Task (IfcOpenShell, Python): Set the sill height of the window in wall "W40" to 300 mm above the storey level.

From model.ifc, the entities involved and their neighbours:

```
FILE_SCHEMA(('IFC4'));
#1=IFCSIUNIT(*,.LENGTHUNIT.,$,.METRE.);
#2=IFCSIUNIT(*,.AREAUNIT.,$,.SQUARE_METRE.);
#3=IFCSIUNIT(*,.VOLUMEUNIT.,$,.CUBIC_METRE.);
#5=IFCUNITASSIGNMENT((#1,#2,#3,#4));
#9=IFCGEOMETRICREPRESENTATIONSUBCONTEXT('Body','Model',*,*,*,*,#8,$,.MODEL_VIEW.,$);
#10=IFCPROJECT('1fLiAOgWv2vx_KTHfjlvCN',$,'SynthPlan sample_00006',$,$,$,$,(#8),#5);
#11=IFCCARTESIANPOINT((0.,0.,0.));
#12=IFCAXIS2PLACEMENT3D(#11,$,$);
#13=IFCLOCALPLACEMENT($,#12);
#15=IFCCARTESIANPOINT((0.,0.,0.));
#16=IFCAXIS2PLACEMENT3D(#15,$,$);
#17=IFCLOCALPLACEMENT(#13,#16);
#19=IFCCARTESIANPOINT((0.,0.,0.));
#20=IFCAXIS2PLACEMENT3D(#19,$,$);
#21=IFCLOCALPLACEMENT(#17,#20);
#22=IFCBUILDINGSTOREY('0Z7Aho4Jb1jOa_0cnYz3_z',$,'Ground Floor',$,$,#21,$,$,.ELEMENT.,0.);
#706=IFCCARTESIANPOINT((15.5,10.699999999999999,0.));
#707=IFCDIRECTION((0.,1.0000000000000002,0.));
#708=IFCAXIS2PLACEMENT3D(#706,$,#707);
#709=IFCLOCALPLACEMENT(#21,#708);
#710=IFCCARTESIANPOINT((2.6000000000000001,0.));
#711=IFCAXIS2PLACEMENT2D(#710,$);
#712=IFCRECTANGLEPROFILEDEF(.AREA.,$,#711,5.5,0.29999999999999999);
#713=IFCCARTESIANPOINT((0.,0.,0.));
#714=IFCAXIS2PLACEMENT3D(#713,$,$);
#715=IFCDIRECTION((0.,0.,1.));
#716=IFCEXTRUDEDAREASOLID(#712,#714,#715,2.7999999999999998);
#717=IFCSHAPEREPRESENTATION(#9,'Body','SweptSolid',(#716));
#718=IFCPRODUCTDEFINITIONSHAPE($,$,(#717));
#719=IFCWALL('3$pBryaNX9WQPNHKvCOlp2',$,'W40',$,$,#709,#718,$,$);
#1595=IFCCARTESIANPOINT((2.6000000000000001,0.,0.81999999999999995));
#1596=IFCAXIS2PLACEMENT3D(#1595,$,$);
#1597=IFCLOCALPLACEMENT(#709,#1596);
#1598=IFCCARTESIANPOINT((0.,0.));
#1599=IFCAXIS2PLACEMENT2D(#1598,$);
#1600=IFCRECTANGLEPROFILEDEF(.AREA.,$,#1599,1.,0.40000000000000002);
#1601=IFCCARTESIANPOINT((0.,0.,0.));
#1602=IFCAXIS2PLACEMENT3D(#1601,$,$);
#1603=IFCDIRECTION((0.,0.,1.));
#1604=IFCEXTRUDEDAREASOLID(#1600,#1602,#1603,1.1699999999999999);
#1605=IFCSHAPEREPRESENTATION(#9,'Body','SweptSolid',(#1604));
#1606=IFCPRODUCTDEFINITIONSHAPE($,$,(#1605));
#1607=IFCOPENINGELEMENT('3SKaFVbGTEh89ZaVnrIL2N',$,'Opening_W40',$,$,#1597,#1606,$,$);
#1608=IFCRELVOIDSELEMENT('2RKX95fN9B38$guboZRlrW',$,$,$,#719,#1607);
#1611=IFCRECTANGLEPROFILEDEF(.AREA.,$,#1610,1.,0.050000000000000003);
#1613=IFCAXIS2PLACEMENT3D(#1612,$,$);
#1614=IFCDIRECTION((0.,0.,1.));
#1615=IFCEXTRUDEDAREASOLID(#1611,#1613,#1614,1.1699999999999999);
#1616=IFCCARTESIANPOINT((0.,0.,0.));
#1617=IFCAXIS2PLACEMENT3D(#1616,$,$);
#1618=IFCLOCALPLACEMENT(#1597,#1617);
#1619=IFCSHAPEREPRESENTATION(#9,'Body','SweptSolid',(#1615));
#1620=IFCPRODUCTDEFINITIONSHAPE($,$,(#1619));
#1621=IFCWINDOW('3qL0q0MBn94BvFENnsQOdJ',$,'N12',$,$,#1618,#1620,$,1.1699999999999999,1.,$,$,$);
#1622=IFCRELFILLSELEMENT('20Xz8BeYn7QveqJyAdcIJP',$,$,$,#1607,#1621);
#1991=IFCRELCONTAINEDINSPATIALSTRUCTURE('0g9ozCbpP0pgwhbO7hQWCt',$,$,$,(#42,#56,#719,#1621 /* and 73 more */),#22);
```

```python
import numpy as np
import ifcopenshell
import ifcopenshell.api.geometry
import ifcopenshell.geom
import ifcopenshell.util.element
import ifcopenshell.util.placement
import ifcopenshell.util.shape
import ifcopenshell.util.unit

model = ifcopenshell.open("model.ifc")
unit_scale = ifcopenshell.util.unit.calculate_unit_scale(model)

window = model.by_guid("3qL0q0MBn94BvFENnsQOdJ")
opening = window.FillsVoids[0].RelatingOpeningElement
storey = ifcopenshell.util.element.get_container(window, ifc_class="IfcBuildingStorey")
level = ifcopenshell.util.placement.get_local_placement(storey.ObjectPlacement)[2, 3]

# The opening's origin need not be at the sill, so measure its lowest point.
shape = ifcopenshell.geom.create_shape(ifcopenshell.geom.settings(), opening)
bottom = ifcopenshell.util.shape.get_shape_bottom_elevation(shape, shape.geometry) / unit_scale
dz = level + 0.3 - bottom

shift = np.array([0.0, 0.0, dz])
# The window is placed relative to its opening, so it follows when the opening moves.
matrix = ifcopenshell.util.placement.get_local_placement(opening.ObjectPlacement)
matrix[:3, 3] += shift
ifcopenshell.api.geometry.edit_object_placement(
    model, product=opening, matrix=matrix, is_si=False, should_transform_children=True
)

print(f"moved by {dz * unit_scale:+.3f} m")

model.write("model_rev.ifc")
```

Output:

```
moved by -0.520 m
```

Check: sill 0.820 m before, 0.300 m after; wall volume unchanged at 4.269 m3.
